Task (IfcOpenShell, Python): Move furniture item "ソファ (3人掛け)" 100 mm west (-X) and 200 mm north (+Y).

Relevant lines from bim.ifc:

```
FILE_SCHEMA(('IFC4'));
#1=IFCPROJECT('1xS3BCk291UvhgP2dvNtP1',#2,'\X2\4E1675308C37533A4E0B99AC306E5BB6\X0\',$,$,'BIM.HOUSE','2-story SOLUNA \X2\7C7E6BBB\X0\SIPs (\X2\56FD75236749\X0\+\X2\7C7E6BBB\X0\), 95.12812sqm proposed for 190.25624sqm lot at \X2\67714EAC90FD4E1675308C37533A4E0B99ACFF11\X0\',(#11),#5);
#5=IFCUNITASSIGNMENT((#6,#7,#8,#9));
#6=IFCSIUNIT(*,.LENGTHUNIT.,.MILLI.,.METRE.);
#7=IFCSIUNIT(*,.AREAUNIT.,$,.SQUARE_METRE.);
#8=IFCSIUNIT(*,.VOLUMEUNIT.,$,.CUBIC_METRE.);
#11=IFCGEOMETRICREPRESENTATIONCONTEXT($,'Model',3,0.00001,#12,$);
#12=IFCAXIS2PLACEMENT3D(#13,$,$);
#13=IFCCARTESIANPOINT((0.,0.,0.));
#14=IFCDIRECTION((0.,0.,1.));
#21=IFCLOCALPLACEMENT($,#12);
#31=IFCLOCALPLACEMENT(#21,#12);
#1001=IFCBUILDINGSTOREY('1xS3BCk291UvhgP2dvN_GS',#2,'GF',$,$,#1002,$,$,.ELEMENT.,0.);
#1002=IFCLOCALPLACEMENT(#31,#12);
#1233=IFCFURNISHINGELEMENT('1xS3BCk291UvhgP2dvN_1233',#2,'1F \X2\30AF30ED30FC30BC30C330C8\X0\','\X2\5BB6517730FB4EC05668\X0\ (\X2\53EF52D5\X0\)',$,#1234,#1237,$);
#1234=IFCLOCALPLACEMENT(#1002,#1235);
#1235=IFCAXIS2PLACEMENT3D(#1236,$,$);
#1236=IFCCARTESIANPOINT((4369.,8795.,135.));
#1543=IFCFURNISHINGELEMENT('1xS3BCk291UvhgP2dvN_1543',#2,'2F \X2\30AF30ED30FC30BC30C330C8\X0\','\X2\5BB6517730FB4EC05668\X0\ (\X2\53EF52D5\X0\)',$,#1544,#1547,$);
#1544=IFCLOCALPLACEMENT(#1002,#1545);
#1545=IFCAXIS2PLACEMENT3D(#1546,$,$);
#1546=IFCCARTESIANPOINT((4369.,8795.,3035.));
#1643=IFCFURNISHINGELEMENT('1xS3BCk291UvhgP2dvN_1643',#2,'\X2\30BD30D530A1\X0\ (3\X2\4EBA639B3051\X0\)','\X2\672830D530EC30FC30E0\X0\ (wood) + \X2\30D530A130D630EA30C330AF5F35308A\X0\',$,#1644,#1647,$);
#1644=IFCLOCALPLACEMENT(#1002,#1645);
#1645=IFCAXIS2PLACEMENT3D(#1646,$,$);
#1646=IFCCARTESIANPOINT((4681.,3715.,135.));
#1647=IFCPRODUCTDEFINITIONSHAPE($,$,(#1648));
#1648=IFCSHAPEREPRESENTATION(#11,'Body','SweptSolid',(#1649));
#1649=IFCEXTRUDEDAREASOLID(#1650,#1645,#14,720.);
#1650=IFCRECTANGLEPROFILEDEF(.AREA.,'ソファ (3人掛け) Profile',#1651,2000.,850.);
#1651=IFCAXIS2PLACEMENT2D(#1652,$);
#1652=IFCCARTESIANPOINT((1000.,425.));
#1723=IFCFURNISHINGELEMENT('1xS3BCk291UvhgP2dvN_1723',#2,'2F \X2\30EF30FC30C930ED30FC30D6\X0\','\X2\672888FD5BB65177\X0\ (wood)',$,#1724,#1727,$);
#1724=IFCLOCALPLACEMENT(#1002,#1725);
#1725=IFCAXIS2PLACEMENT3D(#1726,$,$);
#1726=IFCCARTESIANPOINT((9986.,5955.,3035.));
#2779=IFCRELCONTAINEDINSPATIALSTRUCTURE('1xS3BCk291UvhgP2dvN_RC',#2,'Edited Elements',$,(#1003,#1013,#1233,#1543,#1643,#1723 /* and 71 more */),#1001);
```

```python
import ifcopenshell
import ifcopenshell.api.geometry
import ifcopenshell.util.placement
import ifcopenshell.util.unit

model = ifcopenshell.open("bim.ifc")
unit_scale = ifcopenshell.util.unit.calculate_unit_scale(model)

item = model.by_guid("1xS3BCk291UvhgP2dvN_1643")
matrix = ifcopenshell.util.placement.get_local_placement(item.ObjectPlacement)
matrix[0, 3] -= 0.1 / unit_scale
matrix[1, 3] += 0.2 / unit_scale
ifcopenshell.api.geometry.edit_object_placement(model, product=item, matrix=matrix, is_si=False)

print(ifcopenshell.util.placement.get_local_placement(item.ObjectPlacement).round(3) + 0.0)

model.write("bim_updated.ifc")
```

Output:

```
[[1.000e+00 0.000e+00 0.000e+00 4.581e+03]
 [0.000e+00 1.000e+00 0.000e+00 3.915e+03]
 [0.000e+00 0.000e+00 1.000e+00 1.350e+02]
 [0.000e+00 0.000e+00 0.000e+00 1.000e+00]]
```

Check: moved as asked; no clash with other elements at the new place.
